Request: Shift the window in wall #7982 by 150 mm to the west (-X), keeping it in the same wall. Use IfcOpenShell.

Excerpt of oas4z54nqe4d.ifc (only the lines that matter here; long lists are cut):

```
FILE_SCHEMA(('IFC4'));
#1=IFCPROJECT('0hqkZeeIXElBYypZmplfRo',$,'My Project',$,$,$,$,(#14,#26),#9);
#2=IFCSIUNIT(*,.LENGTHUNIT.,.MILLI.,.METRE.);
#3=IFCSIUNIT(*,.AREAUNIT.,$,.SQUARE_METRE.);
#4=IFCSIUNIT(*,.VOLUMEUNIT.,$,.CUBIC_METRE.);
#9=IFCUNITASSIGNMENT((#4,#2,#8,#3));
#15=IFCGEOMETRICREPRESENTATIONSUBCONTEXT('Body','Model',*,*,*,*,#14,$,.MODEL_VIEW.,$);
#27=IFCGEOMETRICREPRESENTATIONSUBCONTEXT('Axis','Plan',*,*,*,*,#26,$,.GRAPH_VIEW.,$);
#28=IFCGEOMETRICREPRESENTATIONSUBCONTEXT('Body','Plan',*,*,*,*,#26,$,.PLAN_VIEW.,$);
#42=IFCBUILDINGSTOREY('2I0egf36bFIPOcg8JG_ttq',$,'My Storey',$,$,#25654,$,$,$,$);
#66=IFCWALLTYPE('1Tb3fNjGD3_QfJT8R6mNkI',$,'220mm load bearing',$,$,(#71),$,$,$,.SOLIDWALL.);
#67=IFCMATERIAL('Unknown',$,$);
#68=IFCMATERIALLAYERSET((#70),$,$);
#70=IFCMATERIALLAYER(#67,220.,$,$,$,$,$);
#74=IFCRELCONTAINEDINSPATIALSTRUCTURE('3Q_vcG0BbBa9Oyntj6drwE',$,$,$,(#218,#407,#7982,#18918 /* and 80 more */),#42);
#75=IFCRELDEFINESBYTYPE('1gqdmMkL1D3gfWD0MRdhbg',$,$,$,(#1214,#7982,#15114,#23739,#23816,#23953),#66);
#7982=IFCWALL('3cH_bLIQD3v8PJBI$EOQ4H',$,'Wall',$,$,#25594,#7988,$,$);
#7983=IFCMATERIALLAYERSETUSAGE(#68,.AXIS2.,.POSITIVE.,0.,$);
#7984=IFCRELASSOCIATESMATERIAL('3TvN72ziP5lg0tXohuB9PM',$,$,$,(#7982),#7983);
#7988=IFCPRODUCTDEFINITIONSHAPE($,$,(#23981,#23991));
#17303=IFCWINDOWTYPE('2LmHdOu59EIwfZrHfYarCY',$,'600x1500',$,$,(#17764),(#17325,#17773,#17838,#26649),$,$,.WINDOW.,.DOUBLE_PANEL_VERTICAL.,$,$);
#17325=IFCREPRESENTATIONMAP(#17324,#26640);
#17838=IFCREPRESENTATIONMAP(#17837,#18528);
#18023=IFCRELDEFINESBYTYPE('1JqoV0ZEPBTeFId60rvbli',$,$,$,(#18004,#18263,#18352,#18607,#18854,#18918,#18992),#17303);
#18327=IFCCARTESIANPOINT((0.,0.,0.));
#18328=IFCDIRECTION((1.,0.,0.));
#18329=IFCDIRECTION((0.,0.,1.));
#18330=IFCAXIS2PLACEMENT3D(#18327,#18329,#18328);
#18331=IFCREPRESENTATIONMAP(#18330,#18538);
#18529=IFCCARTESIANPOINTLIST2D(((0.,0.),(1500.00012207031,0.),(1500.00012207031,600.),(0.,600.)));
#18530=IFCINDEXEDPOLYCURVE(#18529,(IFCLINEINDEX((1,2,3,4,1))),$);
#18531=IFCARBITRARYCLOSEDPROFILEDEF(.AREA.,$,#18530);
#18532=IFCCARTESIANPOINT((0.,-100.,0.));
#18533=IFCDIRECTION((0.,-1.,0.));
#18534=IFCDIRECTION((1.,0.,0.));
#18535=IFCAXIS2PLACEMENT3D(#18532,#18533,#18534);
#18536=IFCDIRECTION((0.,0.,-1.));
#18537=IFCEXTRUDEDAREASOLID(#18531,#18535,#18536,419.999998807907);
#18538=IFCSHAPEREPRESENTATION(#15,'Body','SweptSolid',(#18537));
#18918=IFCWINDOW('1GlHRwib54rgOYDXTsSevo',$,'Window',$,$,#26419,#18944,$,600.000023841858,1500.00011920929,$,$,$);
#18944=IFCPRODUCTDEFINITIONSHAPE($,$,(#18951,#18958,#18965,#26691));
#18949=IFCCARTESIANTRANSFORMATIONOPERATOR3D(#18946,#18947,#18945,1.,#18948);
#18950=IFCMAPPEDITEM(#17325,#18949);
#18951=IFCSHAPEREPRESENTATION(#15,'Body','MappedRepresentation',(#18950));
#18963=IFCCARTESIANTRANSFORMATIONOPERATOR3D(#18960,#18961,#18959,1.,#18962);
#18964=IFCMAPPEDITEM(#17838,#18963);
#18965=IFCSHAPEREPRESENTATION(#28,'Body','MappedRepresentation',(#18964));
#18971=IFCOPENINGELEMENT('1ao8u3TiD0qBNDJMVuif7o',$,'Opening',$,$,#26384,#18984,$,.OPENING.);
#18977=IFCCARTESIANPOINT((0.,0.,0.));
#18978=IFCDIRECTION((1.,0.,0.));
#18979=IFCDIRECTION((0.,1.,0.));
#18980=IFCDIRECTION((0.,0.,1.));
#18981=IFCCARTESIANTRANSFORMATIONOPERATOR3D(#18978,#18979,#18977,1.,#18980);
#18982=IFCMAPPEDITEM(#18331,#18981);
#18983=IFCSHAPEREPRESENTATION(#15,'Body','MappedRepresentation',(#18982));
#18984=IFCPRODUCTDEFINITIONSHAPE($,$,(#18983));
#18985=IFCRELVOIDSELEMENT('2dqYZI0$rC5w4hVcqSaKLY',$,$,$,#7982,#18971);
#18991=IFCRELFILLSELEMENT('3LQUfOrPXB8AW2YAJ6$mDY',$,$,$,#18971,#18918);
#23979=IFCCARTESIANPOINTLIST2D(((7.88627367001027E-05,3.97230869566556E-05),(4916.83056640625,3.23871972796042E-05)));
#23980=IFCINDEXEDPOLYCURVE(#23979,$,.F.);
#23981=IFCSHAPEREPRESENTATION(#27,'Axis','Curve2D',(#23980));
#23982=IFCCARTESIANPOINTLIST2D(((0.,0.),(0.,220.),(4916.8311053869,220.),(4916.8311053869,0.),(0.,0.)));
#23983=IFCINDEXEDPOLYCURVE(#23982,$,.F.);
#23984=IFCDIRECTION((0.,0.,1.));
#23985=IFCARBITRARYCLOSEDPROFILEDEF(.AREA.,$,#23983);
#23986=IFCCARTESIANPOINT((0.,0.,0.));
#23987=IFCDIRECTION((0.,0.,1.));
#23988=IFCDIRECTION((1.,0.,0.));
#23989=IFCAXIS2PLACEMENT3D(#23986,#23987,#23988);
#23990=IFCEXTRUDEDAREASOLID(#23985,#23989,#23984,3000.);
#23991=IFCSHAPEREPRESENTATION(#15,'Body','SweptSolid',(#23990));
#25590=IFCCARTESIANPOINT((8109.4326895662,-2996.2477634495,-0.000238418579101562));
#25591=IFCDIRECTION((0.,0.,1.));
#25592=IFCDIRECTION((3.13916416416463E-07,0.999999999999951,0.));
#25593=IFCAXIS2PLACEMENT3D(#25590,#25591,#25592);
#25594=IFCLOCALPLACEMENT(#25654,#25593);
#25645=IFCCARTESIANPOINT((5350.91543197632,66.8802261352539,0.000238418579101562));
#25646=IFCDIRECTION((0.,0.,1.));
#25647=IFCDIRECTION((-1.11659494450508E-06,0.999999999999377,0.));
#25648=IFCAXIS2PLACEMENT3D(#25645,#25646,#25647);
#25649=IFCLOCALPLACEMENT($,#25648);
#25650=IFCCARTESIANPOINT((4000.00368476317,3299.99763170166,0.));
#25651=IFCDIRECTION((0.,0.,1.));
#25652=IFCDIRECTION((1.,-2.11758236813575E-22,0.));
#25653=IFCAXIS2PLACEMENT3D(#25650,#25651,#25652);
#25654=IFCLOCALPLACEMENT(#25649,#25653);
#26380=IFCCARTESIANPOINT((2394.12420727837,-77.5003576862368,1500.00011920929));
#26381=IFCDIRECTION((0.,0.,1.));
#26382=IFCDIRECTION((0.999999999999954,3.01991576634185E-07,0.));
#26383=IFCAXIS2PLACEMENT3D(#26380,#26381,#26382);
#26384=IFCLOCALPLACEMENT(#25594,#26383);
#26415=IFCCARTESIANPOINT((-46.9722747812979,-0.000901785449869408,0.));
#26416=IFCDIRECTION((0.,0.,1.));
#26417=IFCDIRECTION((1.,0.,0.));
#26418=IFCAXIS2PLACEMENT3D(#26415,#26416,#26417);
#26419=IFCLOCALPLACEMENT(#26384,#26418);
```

```python
import ifcopenshell
import ifcopenshell.api.geometry
import ifcopenshell.util.placement
import ifcopenshell.util.unit

model = ifcopenshell.open("oas4z54nqe4d.ifc")
unit_scale = ifcopenshell.util.unit.calculate_unit_scale(model)

window = model.by_guid("1GlHRwib54rgOYDXTsSevo")
opening = window.FillsVoids[0].RelatingOpeningElement
wall = opening.VoidsElements[0].RelatingBuildingElement

wall_matrix = ifcopenshell.util.placement.get_local_placement(wall.ObjectPlacement)
shift = wall_matrix[:3, 0] * 0.15 / unit_scale
before = ifcopenshell.util.placement.get_local_placement(window.ObjectPlacement)[:3, 3].copy()

# The window is placed relative to its opening, so it follows when the opening moves.
matrix = ifcopenshell.util.placement.get_local_placement(opening.ObjectPlacement)
matrix[:3, 3] += shift
ifcopenshell.api.geometry.edit_object_placement(
    model, product=opening, matrix=matrix, is_si=False, should_transform_children=True
)

after = ifcopenshell.util.placement.get_local_placement(window.ObjectPlacement)[:3, 3]
print("window moved by", (after - before).round(3) + 0.0)

model.write("oas4z54nqe4d_edited.ifc")
```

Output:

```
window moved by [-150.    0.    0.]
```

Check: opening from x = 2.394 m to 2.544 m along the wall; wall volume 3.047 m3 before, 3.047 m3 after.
